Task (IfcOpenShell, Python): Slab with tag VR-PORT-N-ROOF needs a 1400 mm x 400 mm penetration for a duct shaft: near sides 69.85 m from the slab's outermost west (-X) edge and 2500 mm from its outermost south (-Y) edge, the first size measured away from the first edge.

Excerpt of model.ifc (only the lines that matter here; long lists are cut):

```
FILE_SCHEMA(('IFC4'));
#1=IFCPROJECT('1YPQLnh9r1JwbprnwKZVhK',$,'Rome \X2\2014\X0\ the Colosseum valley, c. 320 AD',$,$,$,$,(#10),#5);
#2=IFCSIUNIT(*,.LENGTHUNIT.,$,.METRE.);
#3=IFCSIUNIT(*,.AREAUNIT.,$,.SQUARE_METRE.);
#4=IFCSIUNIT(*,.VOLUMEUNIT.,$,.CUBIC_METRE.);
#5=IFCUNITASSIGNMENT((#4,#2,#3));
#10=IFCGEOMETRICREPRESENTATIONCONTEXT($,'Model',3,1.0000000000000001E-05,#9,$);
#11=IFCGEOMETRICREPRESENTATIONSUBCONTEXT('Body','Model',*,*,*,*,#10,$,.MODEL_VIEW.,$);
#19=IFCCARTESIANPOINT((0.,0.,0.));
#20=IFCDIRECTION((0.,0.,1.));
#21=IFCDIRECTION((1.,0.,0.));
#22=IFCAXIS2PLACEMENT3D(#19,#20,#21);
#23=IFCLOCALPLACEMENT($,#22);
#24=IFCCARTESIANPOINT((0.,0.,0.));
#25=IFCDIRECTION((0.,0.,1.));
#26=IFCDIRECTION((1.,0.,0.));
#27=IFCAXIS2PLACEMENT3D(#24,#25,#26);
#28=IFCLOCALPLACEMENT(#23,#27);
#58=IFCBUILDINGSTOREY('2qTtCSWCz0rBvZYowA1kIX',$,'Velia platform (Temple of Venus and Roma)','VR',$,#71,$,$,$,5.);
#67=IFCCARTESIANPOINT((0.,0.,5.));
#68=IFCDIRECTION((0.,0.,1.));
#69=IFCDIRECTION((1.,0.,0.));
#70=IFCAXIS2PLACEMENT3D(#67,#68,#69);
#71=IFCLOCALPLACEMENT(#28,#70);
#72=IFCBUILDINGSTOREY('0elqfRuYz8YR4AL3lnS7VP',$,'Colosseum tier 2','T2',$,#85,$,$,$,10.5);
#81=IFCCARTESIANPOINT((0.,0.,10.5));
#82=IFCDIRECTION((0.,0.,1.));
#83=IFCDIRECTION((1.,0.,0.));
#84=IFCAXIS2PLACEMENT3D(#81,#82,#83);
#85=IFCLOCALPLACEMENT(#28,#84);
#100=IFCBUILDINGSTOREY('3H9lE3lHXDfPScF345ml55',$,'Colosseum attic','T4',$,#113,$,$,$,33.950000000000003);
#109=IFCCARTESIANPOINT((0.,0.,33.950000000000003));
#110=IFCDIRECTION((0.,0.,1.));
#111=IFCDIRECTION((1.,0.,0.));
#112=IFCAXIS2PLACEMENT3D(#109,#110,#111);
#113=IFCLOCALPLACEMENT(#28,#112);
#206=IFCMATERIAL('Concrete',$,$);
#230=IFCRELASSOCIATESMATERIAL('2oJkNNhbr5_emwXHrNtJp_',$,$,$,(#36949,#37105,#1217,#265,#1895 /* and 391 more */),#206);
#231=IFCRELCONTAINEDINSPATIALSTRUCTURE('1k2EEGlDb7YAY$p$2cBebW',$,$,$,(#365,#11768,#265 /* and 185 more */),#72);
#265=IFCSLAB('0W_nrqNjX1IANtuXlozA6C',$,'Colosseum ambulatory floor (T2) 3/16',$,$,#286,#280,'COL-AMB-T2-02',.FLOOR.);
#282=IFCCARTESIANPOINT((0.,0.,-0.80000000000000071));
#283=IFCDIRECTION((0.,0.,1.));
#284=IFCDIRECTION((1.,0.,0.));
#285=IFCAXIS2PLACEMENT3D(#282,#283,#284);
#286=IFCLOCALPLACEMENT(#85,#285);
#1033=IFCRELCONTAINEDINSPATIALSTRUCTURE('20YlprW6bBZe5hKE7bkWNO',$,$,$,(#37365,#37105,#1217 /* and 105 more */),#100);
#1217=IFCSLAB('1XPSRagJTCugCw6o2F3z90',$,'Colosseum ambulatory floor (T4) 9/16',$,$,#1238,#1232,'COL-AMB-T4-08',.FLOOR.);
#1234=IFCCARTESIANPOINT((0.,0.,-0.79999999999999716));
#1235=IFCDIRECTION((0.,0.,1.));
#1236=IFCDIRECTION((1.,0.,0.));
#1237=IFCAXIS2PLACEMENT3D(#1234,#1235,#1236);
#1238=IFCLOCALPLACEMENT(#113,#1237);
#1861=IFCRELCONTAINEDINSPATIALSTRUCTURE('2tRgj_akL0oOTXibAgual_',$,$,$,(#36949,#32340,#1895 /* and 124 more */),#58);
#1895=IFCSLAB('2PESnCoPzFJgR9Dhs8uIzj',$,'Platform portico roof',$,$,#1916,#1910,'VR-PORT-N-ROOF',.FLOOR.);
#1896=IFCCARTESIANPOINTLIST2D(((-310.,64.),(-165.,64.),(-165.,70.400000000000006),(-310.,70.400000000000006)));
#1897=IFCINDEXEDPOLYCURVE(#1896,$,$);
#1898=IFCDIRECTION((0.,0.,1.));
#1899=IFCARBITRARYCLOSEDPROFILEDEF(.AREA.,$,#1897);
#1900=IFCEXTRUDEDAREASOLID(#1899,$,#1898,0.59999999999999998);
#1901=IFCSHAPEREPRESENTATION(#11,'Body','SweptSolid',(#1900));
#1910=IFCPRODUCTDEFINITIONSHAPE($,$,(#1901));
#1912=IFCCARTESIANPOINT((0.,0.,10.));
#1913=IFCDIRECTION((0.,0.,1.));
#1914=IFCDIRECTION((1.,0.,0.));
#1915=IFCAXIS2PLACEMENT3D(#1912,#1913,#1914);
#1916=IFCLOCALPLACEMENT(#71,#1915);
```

```python
import numpy as np
import ifcopenshell
import ifcopenshell.api.feature
import ifcopenshell.api.geometry
import ifcopenshell.api.root
import ifcopenshell.geom
import ifcopenshell.util.placement
import ifcopenshell.util.representation
import ifcopenshell.util.shape
import ifcopenshell.util.unit

model = ifcopenshell.open("model.ifc")
unit_scale = ifcopenshell.util.unit.calculate_unit_scale(model)
settings = ifcopenshell.geom.settings()


def volume(element):
    """Net volume in cubic metres, openings subtracted."""
    shape = ifcopenshell.geom.create_shape(settings, element)
    return ifcopenshell.util.shape.get_volume(shape.geometry)


slab = model.by_guid("2PESnCoPzFJgR9Dhs8uIzj")
before = volume(slab)

# Extent in the slab's own axes, in metres. The edges named are its -X and -Y sides.
slab_shape = ifcopenshell.geom.create_shape(settings, slab)
vertices = ifcopenshell.util.shape.get_vertices(slab_shape.geometry)
x_min, y_min, bottom = vertices.min(axis=0)
top = vertices[:, 2].max()

opening = ifcopenshell.api.root.create_entity(model, ifc_class="IfcOpeningElement", name="Duct shaft opening", predefined_type="OPENING")
context = ifcopenshell.util.representation.get_context(model, "Model", "Body", "MODEL_VIEW")
width, depth = 1.4, 0.4
outline = [(0.0, 0.0), (width, 0.0), (width, depth), (0.0, depth), (0.0, 0.0)]
# Overshoot both faces by 50 mm so the cut is clean.
shape = ifcopenshell.api.geometry.add_slab_representation(
    model, context=context, depth=top - bottom + 0.1, polyline=outline
)
ifcopenshell.api.geometry.assign_representation(model, product=opening, representation=shape)

matrix = ifcopenshell.util.placement.get_local_placement(slab.ObjectPlacement)
matrix[:, 3] = matrix @ np.append(np.array([x_min + 69.85, y_min + 2.5, bottom - 0.05]) / unit_scale, 1.0)
ifcopenshell.api.geometry.edit_object_placement(model, product=opening, matrix=matrix, is_si=False)
ifcopenshell.api.feature.add_feature(model, feature=opening, element=slab)

after = volume(slab)

print(f"slab volume {before:.3f} -> {after:.3f} m3")

model.write("model_updated.ifc")
```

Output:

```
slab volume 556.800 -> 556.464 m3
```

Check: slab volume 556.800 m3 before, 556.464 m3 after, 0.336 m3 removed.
